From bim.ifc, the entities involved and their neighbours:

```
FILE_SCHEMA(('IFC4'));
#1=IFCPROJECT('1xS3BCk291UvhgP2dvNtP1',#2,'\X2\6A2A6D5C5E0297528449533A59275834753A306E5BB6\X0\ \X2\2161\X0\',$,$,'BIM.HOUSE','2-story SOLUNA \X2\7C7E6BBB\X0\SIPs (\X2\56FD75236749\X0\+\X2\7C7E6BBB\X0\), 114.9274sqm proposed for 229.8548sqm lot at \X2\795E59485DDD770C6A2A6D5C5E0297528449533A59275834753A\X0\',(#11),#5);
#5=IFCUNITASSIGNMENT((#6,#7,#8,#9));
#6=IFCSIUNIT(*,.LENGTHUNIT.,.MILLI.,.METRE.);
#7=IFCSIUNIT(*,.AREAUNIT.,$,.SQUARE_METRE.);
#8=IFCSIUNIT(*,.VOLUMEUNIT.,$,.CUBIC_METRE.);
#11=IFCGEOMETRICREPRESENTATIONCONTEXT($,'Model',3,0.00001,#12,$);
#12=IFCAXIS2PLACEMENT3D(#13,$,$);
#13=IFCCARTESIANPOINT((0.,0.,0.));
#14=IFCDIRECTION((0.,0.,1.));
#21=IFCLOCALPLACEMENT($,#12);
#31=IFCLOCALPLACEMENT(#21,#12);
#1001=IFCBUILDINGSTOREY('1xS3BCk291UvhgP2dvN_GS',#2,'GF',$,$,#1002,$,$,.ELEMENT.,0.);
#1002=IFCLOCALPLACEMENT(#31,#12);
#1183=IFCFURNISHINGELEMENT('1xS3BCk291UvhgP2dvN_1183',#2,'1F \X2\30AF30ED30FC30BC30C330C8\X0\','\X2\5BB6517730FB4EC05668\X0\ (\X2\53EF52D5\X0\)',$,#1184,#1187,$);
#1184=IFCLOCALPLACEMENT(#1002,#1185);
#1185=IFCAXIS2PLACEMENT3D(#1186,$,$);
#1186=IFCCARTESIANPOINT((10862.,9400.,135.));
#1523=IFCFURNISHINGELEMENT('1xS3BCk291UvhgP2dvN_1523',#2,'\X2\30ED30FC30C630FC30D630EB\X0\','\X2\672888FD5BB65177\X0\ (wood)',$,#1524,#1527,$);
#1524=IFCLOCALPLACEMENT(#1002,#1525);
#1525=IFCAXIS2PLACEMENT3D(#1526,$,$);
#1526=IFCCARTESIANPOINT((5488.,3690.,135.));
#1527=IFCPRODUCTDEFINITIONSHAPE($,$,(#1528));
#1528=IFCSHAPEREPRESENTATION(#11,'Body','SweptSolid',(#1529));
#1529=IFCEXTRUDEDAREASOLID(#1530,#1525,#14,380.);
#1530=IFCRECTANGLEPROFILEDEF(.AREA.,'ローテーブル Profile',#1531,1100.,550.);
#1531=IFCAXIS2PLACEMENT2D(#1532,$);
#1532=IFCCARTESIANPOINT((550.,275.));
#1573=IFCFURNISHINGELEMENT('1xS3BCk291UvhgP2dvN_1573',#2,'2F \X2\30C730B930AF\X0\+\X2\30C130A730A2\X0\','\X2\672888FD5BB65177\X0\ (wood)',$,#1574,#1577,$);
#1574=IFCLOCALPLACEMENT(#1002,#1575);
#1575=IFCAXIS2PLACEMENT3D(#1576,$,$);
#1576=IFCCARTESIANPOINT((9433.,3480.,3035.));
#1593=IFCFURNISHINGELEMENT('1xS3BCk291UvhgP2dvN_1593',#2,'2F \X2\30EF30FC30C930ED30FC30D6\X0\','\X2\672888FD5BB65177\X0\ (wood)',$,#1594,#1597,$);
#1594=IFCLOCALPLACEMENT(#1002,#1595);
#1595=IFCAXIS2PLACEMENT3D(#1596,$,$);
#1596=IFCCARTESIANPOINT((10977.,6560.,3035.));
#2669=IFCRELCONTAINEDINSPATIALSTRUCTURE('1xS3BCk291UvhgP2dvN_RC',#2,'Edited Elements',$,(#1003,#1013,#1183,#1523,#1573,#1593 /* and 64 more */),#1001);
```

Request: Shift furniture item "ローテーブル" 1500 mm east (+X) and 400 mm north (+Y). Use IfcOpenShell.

```python
import ifcopenshell
import ifcopenshell.api.geometry
import ifcopenshell.util.placement
import ifcopenshell.util.unit

model = ifcopenshell.open("bim.ifc")
unit_scale = ifcopenshell.util.unit.calculate_unit_scale(model)

item = model.by_guid("1xS3BCk291UvhgP2dvN_1523")
matrix = ifcopenshell.util.placement.get_local_placement(item.ObjectPlacement)
matrix[0, 3] += 1.5 / unit_scale
matrix[1, 3] += 0.4 / unit_scale
ifcopenshell.api.geometry.edit_object_placement(model, product=item, matrix=matrix, is_si=False)

print(ifcopenshell.util.placement.get_local_placement(item.ObjectPlacement).round(3) + 0.0)

model.write("bim-out.ifc")
```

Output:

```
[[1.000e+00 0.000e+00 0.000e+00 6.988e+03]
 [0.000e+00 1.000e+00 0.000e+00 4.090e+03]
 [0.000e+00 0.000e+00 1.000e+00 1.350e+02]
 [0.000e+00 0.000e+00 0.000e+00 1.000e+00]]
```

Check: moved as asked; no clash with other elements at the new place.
